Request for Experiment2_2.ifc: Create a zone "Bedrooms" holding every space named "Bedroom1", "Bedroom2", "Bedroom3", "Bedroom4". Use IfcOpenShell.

First a look at what the model holds.

```python
import ifcopenshell

model = ifcopenshell.open("Experiment2_2.ifc")
print(model.schema)
seen = {}
for space in model.by_type("IfcSpace"):
    seen[space.LongName] = seen.get(space.LongName, 0) + 1
for name, count in sorted(seen.items(), key=str):
    print(count, "x", name)
print("zones:", [z.Name for z in model.by_type("IfcZone")][:20])
```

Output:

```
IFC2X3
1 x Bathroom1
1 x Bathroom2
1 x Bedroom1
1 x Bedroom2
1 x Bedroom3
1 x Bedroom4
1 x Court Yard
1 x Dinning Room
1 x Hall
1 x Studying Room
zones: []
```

```python
import ifcopenshell
import ifcopenshell.api.group
import ifcopenshell.api.root

model = ifcopenshell.open("Experiment2_2.ifc")

names = {"Bedroom1", "Bedroom2", "Bedroom3", "Bedroom4"}
spaces = [s for s in model.by_type("IfcSpace") if s.LongName in names]

zone = ifcopenshell.api.root.create_entity(model, ifc_class="IfcZone", name="Bedrooms")
ifcopenshell.api.group.assign_group(model, products=spaces, group=zone)
print(len(spaces), "spaces in", zone.Name)

model.write("Experiment2_2_v2.ifc")
```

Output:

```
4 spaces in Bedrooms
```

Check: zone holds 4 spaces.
